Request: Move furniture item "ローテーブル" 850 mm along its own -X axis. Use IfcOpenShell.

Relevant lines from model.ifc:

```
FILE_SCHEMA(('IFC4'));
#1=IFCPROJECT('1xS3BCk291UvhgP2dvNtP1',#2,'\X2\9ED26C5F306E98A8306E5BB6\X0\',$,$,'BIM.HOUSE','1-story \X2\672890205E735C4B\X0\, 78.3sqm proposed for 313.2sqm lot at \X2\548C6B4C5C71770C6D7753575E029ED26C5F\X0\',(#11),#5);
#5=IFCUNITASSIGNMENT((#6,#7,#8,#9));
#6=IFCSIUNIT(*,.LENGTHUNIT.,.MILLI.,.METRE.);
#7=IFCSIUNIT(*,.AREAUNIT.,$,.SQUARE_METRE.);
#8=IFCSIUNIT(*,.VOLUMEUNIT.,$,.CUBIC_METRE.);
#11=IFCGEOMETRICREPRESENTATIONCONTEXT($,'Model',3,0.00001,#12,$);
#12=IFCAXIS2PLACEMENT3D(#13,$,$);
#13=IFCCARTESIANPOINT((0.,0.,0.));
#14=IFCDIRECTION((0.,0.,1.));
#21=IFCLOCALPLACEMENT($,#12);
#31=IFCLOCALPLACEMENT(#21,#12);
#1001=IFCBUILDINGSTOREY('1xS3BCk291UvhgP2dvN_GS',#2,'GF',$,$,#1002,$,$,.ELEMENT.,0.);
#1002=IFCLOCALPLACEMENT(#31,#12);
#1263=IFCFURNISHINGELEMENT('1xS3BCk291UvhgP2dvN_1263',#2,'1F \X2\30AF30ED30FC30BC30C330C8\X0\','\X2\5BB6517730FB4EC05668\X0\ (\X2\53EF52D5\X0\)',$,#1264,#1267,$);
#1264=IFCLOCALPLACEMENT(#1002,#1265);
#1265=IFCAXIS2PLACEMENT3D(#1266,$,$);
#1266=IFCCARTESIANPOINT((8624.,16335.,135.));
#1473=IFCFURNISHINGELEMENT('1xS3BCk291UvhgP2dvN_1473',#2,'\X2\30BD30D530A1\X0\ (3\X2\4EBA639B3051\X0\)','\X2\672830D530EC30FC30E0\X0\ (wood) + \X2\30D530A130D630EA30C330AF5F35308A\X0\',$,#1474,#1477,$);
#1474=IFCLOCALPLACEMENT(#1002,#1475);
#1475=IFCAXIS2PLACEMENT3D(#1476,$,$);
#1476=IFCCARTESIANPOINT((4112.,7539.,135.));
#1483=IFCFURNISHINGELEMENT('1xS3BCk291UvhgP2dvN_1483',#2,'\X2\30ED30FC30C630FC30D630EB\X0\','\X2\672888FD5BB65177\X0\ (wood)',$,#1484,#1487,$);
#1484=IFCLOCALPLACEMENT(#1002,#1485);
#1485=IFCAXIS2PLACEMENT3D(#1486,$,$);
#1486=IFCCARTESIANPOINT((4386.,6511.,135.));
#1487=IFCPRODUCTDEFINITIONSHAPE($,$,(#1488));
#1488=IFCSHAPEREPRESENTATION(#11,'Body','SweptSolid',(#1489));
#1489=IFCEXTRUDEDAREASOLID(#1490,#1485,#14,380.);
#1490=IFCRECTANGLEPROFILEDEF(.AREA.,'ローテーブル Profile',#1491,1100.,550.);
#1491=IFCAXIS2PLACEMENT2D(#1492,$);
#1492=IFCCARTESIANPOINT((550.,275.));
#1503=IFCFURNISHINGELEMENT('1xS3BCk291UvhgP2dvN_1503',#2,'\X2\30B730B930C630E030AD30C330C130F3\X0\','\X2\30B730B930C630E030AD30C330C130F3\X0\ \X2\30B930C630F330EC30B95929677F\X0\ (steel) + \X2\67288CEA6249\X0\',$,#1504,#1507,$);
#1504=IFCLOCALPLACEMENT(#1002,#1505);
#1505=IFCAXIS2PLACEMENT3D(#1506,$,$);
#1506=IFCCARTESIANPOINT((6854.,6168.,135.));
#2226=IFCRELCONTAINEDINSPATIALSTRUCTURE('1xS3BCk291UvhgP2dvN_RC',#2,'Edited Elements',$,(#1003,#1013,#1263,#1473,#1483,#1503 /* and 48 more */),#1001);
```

```python
import ifcopenshell
import ifcopenshell.api.geometry
import ifcopenshell.util.placement
import ifcopenshell.util.unit

model = ifcopenshell.open("model.ifc")
unit_scale = ifcopenshell.util.unit.calculate_unit_scale(model)

item = model.by_guid("1xS3BCk291UvhgP2dvN_1483")
matrix = ifcopenshell.util.placement.get_local_placement(item.ObjectPlacement)
matrix[:3, 3] -= matrix[:3, 0] * 0.85 / unit_scale
ifcopenshell.api.geometry.edit_object_placement(model, product=item, matrix=matrix, is_si=False)

print(ifcopenshell.util.placement.get_local_placement(item.ObjectPlacement).round(3) + 0.0)

model.write("model_v2.ifc")
```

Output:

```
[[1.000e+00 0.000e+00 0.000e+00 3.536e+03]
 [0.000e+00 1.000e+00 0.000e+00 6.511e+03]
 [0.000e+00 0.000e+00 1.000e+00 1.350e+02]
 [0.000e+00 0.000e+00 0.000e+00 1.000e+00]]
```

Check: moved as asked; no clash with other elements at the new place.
